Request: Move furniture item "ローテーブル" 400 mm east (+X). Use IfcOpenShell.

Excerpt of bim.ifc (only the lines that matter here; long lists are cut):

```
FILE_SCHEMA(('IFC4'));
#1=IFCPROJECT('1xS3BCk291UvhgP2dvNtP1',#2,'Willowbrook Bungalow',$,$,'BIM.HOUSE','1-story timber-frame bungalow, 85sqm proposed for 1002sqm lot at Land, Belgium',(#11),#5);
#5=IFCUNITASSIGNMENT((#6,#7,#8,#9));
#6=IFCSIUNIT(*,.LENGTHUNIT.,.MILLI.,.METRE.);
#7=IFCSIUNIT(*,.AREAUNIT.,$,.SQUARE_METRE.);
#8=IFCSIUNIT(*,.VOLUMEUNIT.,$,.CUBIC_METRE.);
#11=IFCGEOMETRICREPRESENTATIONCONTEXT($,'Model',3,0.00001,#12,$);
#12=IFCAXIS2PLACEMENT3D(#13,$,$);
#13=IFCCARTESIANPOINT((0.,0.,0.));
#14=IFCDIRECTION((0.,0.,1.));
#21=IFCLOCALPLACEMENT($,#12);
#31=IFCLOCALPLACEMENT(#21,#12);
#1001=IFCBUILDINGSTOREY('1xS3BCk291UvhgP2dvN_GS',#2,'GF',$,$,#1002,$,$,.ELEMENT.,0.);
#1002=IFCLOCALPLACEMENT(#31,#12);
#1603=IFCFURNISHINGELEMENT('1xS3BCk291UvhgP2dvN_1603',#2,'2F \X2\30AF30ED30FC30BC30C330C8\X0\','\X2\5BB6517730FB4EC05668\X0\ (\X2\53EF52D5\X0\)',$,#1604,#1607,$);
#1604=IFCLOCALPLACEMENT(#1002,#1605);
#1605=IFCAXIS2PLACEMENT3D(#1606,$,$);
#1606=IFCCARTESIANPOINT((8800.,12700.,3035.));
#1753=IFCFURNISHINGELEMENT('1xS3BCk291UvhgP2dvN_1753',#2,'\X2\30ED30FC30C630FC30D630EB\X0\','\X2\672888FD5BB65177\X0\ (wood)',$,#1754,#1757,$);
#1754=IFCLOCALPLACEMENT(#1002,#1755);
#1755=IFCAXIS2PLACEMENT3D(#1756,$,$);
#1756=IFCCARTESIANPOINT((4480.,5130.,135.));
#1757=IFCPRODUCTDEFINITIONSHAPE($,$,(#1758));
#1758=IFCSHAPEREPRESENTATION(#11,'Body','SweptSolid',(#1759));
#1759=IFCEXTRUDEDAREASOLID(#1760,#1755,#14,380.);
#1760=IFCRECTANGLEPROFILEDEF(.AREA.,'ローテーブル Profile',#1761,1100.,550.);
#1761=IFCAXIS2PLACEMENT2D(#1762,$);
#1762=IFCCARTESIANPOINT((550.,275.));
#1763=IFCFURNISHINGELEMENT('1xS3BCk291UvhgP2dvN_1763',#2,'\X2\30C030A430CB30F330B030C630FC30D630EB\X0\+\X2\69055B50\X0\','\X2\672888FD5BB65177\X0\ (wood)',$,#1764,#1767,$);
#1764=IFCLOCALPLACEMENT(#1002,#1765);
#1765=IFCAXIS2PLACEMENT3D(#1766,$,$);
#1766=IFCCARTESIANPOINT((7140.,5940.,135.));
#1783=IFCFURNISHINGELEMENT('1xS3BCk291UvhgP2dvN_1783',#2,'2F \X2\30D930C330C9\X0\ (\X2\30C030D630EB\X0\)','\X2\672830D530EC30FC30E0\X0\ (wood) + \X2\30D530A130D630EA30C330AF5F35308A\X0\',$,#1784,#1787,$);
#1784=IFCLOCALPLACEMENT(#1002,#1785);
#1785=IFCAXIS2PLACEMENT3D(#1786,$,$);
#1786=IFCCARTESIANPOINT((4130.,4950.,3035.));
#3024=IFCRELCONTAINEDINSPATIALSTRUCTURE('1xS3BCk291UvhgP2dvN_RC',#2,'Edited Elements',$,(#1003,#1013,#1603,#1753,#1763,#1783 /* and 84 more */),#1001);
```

```python
import ifcopenshell
import ifcopenshell.api.geometry
import ifcopenshell.util.placement
import ifcopenshell.util.unit

model = ifcopenshell.open("bim.ifc")
unit_scale = ifcopenshell.util.unit.calculate_unit_scale(model)

item = model.by_id(1753)
matrix = ifcopenshell.util.placement.get_local_placement(item.ObjectPlacement)
matrix[0, 3] += 0.4 / unit_scale
ifcopenshell.api.geometry.edit_object_placement(model, product=item, matrix=matrix, is_si=False)

print(ifcopenshell.util.placement.get_local_placement(item.ObjectPlacement).round(3) + 0.0)

model.write("bim_updated.ifc")
```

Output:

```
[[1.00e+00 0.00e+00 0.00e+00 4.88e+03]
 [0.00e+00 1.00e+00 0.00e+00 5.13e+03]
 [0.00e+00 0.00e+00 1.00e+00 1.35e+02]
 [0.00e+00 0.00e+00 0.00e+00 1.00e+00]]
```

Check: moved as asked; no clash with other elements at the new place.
